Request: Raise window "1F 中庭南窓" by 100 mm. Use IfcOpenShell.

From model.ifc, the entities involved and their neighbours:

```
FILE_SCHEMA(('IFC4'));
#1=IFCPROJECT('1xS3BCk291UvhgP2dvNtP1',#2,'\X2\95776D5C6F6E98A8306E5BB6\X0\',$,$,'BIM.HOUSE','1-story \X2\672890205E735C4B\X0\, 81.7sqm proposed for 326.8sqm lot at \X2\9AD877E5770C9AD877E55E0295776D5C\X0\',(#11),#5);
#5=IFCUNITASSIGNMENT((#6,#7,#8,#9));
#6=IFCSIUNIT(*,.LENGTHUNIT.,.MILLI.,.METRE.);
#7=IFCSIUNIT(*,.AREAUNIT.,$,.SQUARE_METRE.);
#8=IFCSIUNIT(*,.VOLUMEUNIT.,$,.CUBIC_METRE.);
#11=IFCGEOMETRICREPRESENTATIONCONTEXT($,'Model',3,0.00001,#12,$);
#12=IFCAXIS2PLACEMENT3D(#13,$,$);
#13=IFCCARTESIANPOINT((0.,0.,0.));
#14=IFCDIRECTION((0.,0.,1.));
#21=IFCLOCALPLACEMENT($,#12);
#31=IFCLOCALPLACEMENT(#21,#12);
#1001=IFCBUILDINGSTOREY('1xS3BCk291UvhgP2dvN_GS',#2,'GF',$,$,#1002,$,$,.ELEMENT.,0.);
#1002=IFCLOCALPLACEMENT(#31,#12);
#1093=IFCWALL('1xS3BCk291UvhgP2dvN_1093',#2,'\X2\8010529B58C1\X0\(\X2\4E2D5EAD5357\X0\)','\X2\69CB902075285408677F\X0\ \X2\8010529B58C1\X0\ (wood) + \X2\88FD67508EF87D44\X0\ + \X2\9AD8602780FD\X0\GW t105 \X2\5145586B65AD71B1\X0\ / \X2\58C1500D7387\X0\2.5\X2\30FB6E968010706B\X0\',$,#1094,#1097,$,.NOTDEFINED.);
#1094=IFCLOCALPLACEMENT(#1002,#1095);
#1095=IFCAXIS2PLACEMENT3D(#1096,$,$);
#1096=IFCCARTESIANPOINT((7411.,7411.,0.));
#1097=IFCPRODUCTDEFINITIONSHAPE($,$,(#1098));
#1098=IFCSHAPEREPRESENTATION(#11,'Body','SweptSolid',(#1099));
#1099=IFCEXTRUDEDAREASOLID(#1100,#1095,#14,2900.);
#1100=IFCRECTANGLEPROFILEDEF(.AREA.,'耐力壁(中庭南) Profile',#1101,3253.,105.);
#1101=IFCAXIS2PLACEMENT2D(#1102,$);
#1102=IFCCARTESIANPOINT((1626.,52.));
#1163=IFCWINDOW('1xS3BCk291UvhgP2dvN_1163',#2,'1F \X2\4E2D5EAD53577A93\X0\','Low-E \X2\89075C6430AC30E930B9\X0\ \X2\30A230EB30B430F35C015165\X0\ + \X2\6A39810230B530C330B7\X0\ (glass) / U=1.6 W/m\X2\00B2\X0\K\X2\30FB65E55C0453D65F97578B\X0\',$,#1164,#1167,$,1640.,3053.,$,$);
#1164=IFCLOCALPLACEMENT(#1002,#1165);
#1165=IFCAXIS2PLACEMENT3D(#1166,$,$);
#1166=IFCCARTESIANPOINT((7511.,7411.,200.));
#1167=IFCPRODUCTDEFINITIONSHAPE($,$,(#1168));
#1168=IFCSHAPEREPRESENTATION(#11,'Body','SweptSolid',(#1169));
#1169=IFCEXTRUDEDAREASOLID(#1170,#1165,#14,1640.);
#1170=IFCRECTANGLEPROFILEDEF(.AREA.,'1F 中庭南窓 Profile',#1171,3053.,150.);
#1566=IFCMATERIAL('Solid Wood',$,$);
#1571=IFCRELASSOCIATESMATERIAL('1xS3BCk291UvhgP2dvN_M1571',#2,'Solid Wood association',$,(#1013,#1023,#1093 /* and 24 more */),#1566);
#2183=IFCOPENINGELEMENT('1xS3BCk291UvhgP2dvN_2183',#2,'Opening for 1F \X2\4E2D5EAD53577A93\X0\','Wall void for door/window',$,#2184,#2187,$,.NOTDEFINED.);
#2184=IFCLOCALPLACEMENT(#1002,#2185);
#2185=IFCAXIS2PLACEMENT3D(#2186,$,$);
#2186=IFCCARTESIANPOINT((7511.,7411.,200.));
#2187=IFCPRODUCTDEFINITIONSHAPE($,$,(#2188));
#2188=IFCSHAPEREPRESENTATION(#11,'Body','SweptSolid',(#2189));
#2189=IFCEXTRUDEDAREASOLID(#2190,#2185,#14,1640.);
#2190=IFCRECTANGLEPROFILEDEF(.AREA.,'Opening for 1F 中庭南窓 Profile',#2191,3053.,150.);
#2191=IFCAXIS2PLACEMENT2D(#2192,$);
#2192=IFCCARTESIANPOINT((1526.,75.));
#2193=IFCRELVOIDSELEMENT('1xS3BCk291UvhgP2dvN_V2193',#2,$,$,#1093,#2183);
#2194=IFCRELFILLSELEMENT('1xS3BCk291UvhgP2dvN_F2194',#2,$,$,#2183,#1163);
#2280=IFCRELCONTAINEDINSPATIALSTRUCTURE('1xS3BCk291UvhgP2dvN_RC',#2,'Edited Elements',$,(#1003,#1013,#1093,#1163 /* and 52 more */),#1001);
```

```python
import numpy as np
import ifcopenshell
import ifcopenshell.api.geometry
import ifcopenshell.util.placement
import ifcopenshell.util.unit

model = ifcopenshell.open("model.ifc")
unit_scale = ifcopenshell.util.unit.calculate_unit_scale(model)

window = model.by_guid("1xS3BCk291UvhgP2dvN_1163")
opening = window.FillsVoids[0].RelatingOpeningElement
dz = 0.1 / unit_scale

shift = np.array([0.0, 0.0, dz])
# The window is not placed relative to its opening, so move both.
for product in (opening, window):
    matrix = ifcopenshell.util.placement.get_local_placement(product.ObjectPlacement)
    matrix[:3, 3] += shift
    ifcopenshell.api.geometry.edit_object_placement(model, product=product, matrix=matrix, is_si=False)

print(f"moved by {dz * unit_scale:+.3f} m")

model.write("model_rev.ifc")
```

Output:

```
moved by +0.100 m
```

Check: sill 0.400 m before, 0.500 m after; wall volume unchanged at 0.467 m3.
